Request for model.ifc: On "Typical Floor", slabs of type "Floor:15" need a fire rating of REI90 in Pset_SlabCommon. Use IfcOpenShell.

First a look at what the model holds.

```python
import ifcopenshell
import ifcopenshell.util.element

model = ifcopenshell.open("model.ifc")
print(model.schema)
storey = next(s for s in model.by_type("IfcBuildingStorey") if s.Name == "Typical Floor")
slabs = [e for e in ifcopenshell.util.element.get_decomposition(storey) if e.is_a("IfcSlab")]
seen = {}
for e in slabs:
    element_type = ifcopenshell.util.element.get_type(e)
    key = (element_type.Name if element_type != e and element_type else None, ifcopenshell.util.element.get_pset(e, "Pset_SlabCommon", "FireRating"))
    seen[key] = seen.get(key, 0) + 1
for (name, value), count in sorted(seen.items(), key=str):
    print(count, "x", name, "|", value)
```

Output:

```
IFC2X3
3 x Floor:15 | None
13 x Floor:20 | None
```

```python
import ifcopenshell
import ifcopenshell.api.pset
import ifcopenshell.util.element

model = ifcopenshell.open("model.ifc")

storey = next(s for s in model.by_type("IfcBuildingStorey") if s.Name == "Typical Floor")
slabs = [e for e in ifcopenshell.util.element.get_decomposition(storey) if e.is_a("IfcSlab")]

count = 0
for e in slabs:
    element_type = ifcopenshell.util.element.get_type(e)
    if element_type in (None, e) or element_type.Name != "Floor:15":
        continue
    # add_pset returns the element's existing set when there is one.
    pset = ifcopenshell.api.pset.add_pset(model, product=e, name="Pset_SlabCommon")
    ifcopenshell.api.pset.edit_pset(model, pset=pset, properties={"FireRating": "REI90"})
    count += 1

print(count, "slabs updated")

model.write("model_rev.ifc")
```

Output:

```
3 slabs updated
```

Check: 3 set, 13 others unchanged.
